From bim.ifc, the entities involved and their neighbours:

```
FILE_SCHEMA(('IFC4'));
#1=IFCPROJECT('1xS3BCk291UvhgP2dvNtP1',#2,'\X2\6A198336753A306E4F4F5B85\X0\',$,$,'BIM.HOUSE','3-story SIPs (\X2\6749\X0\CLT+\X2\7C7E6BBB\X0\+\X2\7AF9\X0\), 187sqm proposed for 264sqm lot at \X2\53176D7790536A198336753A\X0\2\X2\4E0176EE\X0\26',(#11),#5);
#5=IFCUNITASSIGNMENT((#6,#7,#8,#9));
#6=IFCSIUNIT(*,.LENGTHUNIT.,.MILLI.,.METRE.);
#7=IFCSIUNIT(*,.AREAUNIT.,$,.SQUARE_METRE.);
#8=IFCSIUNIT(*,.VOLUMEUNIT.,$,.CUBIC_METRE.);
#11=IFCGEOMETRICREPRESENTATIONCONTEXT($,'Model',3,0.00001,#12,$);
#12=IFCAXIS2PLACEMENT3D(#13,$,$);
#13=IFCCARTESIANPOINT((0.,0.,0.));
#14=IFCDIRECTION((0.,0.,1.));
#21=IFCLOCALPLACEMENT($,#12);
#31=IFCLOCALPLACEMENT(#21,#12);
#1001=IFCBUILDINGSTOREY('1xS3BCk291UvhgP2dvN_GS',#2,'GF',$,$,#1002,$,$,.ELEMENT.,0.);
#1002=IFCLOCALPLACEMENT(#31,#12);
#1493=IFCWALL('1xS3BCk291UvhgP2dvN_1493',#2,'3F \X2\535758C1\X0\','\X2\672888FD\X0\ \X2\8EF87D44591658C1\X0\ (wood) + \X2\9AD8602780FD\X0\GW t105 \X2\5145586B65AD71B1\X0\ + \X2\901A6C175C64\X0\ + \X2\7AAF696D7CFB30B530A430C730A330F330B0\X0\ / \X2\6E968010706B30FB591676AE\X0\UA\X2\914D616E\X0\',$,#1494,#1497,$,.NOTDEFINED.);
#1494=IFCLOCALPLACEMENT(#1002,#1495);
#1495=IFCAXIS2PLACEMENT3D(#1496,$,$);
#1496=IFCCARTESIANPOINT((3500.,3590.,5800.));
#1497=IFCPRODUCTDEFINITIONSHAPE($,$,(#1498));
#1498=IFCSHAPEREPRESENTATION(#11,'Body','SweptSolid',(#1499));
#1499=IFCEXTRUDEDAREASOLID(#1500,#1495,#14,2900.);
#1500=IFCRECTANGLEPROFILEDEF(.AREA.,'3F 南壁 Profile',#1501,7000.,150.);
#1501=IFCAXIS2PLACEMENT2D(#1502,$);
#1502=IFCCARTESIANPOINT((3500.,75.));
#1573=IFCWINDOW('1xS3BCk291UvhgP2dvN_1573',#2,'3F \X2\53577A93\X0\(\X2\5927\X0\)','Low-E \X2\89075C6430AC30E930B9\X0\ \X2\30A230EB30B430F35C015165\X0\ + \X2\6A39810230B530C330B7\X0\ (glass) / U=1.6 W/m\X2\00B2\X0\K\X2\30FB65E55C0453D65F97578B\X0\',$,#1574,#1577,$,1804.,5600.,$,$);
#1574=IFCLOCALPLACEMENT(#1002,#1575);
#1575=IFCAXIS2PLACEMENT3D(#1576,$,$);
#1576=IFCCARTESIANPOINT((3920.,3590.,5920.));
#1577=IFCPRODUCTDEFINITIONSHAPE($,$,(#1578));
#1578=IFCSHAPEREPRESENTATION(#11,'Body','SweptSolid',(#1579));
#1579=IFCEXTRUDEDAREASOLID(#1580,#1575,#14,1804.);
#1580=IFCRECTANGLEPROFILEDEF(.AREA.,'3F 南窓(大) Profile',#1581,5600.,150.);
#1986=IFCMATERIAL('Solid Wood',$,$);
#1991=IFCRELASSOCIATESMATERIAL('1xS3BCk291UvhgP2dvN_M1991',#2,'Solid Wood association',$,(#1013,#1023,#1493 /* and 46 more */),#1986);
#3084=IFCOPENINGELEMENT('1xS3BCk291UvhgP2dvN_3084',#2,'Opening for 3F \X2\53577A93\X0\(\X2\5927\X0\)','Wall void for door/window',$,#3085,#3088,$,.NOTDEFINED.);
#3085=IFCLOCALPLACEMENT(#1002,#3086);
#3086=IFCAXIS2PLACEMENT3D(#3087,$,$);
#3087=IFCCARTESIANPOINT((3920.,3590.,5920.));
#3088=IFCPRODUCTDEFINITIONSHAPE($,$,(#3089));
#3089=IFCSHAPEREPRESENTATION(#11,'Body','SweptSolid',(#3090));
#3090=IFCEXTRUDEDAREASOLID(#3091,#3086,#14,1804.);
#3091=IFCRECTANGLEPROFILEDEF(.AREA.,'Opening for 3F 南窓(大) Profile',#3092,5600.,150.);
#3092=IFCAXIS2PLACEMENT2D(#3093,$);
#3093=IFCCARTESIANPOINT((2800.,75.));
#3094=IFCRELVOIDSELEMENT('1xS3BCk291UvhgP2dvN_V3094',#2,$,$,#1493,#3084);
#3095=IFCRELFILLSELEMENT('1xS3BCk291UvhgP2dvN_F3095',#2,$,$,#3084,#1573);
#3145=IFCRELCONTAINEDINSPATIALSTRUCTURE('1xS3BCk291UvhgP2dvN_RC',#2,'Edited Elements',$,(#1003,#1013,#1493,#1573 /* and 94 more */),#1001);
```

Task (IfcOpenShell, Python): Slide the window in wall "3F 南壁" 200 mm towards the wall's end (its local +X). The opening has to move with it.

```python
import ifcopenshell
import ifcopenshell.api.geometry
import ifcopenshell.util.placement

model = ifcopenshell.open("bim.ifc")

window = model.by_guid("1xS3BCk291UvhgP2dvN_1573")
opening = window.FillsVoids[0].RelatingOpeningElement
wall = opening.VoidsElements[0].RelatingBuildingElement

wall_matrix = ifcopenshell.util.placement.get_local_placement(wall.ObjectPlacement)
shift = wall_matrix[:3, 0] * 200.0
before = ifcopenshell.util.placement.get_local_placement(window.ObjectPlacement)[:3, 3].copy()

# The window is not placed relative to its opening, so move both.
for product in (opening, window):
    matrix = ifcopenshell.util.placement.get_local_placement(product.ObjectPlacement)
    matrix[:3, 3] += shift
    ifcopenshell.api.geometry.edit_object_placement(model, product=product, matrix=matrix, is_si=False)

after = ifcopenshell.util.placement.get_local_placement(window.ObjectPlacement)[:3, 3]
print("window moved by", (after - before).round(3) + 0.0)

model.write("bim_v2.ifc")
```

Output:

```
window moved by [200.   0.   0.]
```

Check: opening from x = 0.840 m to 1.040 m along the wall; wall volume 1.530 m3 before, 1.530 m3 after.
